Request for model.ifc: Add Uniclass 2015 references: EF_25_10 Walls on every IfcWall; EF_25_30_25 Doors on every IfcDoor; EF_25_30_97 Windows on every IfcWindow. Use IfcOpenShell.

First a look at what the model holds.

```python
import ifcopenshell

model = ifcopenshell.open("model.ifc")
print(model.schema)
print("classifications:", [c.Name for c in model.by_type("IfcClassification")])
for ifc_class in ("IfcDoor", "IfcRoof", "IfcStair", "IfcWall", "IfcWindow"):
    print(ifc_class, len(model.by_type(ifc_class)))
```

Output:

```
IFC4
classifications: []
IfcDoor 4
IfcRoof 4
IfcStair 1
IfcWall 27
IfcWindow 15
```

```python
import ifcopenshell
import ifcopenshell.api.classification

model = ifcopenshell.open("model.ifc")

system = ifcopenshell.api.classification.add_classification(model, classification="Uniclass 2015")

codes = {
    "IfcWall": ("EF_25_10", "Walls"),
    "IfcDoor": ("EF_25_30_25", "Doors"),
    "IfcWindow": ("EF_25_30_97", "Windows"),
}
for ifc_class, (code, name) in codes.items():
    products = model.by_type(ifc_class)
    ifcopenshell.api.classification.add_reference(
        model, products=products, classification=system, identification=code, name=name
    )
    print(code, len(products))

model.write("model_v2.ifc")
```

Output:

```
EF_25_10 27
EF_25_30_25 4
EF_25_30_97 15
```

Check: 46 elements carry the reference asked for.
